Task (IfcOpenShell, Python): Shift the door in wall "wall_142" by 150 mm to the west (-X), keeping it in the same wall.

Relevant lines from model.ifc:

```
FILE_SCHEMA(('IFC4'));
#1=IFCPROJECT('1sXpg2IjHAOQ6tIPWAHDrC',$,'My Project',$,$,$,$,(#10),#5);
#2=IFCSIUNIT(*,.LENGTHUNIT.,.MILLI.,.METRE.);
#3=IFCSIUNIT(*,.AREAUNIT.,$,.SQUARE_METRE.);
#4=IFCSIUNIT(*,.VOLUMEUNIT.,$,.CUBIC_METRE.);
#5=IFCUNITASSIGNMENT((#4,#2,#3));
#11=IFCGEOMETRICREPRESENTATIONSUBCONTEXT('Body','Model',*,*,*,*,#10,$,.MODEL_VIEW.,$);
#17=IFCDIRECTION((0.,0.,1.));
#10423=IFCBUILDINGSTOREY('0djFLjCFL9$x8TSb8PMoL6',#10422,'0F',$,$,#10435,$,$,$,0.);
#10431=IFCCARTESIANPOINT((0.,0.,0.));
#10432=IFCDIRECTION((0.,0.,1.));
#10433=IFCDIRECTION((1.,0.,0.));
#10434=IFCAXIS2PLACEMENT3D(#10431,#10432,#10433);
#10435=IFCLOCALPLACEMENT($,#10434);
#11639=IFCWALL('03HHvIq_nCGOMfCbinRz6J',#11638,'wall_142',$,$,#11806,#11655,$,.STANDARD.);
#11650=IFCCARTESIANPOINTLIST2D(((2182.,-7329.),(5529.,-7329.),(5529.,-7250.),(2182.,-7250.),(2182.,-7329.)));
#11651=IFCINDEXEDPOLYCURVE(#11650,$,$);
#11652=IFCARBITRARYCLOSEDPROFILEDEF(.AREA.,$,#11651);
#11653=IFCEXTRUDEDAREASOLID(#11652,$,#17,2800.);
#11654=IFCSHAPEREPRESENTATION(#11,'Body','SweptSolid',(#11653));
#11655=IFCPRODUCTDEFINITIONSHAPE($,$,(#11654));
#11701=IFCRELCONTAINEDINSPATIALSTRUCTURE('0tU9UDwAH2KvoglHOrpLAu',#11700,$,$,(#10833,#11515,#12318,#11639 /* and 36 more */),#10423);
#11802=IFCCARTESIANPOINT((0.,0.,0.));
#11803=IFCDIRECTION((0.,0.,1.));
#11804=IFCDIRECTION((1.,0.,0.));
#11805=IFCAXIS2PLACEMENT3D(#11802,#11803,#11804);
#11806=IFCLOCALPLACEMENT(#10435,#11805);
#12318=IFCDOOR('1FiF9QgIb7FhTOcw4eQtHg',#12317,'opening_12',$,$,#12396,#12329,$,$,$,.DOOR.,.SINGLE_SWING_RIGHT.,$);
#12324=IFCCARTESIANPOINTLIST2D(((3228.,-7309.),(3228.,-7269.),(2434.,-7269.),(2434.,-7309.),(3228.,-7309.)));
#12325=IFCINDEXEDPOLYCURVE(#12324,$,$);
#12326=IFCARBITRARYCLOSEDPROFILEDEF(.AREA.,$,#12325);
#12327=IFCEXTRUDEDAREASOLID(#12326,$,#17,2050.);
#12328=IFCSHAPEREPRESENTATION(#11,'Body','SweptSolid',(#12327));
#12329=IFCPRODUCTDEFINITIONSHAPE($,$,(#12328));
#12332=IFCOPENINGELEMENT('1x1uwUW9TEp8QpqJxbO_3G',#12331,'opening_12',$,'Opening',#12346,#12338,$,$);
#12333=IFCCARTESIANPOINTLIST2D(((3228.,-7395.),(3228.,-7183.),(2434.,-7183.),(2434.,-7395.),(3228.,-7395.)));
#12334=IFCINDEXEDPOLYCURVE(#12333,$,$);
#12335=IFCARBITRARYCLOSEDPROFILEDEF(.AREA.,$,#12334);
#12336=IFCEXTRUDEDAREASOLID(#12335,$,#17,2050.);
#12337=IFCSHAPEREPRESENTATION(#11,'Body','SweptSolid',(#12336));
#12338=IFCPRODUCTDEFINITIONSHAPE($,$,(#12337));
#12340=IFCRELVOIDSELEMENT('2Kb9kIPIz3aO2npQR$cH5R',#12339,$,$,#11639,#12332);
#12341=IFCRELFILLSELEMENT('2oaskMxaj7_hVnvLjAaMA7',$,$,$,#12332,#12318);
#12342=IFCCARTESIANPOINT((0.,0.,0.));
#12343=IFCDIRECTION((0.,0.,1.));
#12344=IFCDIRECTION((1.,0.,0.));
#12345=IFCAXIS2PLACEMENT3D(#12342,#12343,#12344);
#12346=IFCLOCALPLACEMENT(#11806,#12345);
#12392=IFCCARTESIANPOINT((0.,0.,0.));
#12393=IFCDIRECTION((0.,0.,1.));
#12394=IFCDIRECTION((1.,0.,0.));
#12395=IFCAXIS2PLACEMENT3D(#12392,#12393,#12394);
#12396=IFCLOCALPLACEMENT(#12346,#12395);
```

```python
import ifcopenshell
import ifcopenshell.api.geometry
import ifcopenshell.util.placement
import ifcopenshell.util.unit

model = ifcopenshell.open("model.ifc")
unit_scale = ifcopenshell.util.unit.calculate_unit_scale(model)

door = model.by_id(12318)
opening = door.FillsVoids[0].RelatingOpeningElement
wall = opening.VoidsElements[0].RelatingBuildingElement

wall_matrix = ifcopenshell.util.placement.get_local_placement(wall.ObjectPlacement)
shift = wall_matrix[:3, 0] * -0.15 / unit_scale
before = ifcopenshell.util.placement.get_local_placement(door.ObjectPlacement)[:3, 3].copy()

# The door is placed relative to its opening, so it follows when the opening moves.
matrix = ifcopenshell.util.placement.get_local_placement(opening.ObjectPlacement)
matrix[:3, 3] += shift
ifcopenshell.api.geometry.edit_object_placement(
    model, product=opening, matrix=matrix, is_si=False, should_transform_children=True
)

after = ifcopenshell.util.placement.get_local_placement(door.ObjectPlacement)[:3, 3]
print("door moved by", (after - before).round(3) + 0.0)

model.write("model_edited.ifc")
```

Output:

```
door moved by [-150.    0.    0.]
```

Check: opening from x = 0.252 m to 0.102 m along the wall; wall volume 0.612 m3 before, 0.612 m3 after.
